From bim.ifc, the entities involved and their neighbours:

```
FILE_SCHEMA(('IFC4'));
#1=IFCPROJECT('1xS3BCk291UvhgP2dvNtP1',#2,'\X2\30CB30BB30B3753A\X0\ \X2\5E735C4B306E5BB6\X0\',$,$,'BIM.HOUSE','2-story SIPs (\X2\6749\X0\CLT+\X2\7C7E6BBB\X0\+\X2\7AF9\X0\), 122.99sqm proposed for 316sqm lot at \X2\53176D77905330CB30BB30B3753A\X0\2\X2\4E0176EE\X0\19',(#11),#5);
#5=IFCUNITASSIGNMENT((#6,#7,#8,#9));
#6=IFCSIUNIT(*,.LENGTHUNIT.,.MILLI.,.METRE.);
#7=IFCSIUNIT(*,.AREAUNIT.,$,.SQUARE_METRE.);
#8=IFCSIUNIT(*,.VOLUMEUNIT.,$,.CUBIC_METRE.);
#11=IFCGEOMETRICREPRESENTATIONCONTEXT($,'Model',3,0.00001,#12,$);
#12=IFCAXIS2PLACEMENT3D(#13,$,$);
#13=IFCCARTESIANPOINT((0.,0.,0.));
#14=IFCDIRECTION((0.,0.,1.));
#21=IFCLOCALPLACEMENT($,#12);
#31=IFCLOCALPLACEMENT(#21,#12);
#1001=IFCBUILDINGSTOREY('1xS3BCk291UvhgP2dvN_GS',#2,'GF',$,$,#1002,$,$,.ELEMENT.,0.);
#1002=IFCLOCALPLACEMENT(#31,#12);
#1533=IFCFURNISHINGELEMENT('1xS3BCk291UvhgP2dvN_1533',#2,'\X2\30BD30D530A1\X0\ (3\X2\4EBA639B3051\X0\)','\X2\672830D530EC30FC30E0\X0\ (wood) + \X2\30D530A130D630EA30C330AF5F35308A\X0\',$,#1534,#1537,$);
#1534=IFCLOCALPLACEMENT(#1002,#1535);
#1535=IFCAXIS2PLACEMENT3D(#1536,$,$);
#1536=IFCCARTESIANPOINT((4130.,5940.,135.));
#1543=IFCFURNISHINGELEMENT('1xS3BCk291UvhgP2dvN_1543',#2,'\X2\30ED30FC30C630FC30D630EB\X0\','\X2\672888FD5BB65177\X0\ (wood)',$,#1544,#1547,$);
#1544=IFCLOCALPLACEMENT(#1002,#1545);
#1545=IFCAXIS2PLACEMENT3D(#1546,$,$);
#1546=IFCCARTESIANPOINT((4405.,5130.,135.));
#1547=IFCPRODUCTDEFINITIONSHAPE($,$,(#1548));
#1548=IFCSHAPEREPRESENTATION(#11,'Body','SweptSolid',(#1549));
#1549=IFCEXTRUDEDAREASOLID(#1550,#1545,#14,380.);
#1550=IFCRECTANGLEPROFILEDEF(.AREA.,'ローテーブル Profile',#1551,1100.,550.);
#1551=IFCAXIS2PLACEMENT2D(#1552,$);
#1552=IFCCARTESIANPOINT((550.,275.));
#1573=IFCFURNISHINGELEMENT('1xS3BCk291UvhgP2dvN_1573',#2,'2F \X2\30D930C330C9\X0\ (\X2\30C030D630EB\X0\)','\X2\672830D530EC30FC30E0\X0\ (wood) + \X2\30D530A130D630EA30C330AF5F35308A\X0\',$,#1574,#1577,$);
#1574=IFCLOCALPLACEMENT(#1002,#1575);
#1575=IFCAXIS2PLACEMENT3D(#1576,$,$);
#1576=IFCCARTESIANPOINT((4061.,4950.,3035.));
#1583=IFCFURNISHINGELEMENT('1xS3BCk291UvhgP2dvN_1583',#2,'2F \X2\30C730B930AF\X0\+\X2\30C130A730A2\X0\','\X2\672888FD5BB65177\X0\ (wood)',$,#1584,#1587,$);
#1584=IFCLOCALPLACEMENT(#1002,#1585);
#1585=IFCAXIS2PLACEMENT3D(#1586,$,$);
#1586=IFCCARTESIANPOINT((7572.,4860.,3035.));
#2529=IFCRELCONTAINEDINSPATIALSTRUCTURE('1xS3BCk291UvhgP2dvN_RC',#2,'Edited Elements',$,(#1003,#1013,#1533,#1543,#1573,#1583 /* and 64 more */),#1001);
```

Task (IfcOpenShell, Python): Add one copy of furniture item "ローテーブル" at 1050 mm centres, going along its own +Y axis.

```python
import ifcopenshell
import ifcopenshell.api.geometry
import ifcopenshell.api.root
import ifcopenshell.util.element
import ifcopenshell.util.placement
import ifcopenshell.util.unit

model = ifcopenshell.open("bim.ifc")
unit_scale = ifcopenshell.util.unit.calculate_unit_scale(model)


def reuse_history(source, copy):
    """copy_class also copies each property set's owner history, people and application; keep the originals."""
    for rel in copy.IsDefinedBy:
        if rel.is_a("IfcRelDefinesByProperties") and (history := rel.RelatingPropertyDefinition.OwnerHistory):
            rel.RelatingPropertyDefinition.OwnerHistory = source.OwnerHistory
            ifcopenshell.util.element.remove_deep2(model, history)


source = model.by_guid("1xS3BCk291UvhgP2dvN_1543")
base = ifcopenshell.util.placement.get_local_placement(source.ObjectPlacement)
step = base[:3, 1] * 1.05 / unit_scale

for i in range(1, 2):
    copy = ifcopenshell.api.root.copy_class(model, product=source)
    copy.Representation = ifcopenshell.util.element.copy_deep(
        model, source.Representation, exclude=["IfcGeometricRepresentationContext", "IfcRepresentationMap"]
    )
    reuse_history(source, copy)
    matrix = base.copy()
    matrix[:3, 3] += i * step
    print("added at", matrix[:3, 3].round(3) + 0.0)
    ifcopenshell.api.geometry.edit_object_placement(model, product=copy, matrix=matrix, is_si=False)

model.write("bim_rev.ifc")
```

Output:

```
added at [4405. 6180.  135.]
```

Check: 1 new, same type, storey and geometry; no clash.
